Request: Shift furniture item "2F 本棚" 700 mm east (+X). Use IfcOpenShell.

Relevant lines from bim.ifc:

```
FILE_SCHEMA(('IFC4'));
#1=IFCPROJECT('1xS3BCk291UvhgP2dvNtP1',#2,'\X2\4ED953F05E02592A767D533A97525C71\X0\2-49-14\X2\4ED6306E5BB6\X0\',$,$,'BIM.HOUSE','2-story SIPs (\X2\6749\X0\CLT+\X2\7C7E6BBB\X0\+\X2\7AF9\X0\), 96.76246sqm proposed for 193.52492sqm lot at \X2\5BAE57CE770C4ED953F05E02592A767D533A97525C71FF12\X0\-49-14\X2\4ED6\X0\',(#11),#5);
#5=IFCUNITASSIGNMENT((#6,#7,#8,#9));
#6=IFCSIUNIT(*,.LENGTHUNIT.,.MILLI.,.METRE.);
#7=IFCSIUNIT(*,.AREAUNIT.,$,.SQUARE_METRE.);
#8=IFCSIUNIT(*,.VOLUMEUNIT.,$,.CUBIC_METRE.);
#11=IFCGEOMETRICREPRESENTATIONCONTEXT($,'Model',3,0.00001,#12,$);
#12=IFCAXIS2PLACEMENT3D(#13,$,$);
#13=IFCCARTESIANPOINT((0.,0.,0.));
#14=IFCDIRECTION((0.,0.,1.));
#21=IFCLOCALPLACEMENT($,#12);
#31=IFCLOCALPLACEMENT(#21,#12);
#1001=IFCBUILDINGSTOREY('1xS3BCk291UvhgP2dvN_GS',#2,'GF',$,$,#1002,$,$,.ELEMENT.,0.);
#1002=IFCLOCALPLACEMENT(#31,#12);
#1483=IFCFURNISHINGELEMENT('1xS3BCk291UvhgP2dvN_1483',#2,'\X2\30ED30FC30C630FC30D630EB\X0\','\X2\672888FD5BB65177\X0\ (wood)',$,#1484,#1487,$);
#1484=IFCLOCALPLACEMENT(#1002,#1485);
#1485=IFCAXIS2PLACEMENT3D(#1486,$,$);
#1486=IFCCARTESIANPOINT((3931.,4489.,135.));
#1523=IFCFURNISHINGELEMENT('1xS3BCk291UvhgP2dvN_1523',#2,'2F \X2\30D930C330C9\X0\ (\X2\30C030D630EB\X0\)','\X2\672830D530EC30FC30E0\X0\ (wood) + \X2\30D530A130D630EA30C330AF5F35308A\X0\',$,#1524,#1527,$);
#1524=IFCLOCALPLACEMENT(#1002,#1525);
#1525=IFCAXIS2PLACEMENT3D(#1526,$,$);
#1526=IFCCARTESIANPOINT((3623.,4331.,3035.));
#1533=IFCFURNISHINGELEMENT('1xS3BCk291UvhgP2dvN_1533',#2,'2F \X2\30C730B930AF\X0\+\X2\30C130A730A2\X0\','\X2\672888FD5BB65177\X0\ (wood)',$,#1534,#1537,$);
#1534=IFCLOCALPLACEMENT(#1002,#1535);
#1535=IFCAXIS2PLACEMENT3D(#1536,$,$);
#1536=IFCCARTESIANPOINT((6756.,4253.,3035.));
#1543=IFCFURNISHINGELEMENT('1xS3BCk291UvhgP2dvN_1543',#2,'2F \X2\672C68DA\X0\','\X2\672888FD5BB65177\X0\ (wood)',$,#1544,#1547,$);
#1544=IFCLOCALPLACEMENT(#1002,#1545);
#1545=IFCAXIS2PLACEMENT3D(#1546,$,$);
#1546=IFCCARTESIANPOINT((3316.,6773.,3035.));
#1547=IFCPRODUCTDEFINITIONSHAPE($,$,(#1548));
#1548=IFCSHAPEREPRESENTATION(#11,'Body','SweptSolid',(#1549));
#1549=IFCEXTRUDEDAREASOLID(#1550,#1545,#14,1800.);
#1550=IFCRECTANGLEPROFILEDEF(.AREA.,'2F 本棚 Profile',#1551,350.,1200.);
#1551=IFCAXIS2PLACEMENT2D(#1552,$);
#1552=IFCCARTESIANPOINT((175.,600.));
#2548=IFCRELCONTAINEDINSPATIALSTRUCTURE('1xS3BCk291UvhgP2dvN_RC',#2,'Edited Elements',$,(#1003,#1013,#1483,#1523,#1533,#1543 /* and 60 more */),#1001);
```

```python
import ifcopenshell
import ifcopenshell.api.geometry
import ifcopenshell.util.placement
import ifcopenshell.util.unit

model = ifcopenshell.open("bim.ifc")
unit_scale = ifcopenshell.util.unit.calculate_unit_scale(model)

item = model.by_guid("1xS3BCk291UvhgP2dvN_1543")
matrix = ifcopenshell.util.placement.get_local_placement(item.ObjectPlacement)
matrix[0, 3] += 0.7 / unit_scale
ifcopenshell.api.geometry.edit_object_placement(model, product=item, matrix=matrix, is_si=False)

print(ifcopenshell.util.placement.get_local_placement(item.ObjectPlacement).round(3) + 0.0)

model.write("bim_updated.ifc")
```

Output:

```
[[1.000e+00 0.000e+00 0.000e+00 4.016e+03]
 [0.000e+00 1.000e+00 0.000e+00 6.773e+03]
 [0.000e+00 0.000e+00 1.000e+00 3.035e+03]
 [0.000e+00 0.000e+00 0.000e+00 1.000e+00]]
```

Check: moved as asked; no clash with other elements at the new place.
